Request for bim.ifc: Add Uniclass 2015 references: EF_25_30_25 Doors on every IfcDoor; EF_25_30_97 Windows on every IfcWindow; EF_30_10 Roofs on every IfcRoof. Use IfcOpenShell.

First a look at what the model holds.

```python
import ifcopenshell

model = ifcopenshell.open("bim.ifc")
print(model.schema)
print("classifications:", [c.Name for c in model.by_type("IfcClassification")])
for ifc_class in ("IfcDoor", "IfcRoof", "IfcStair", "IfcWall", "IfcWindow"):
    print(ifc_class, len(model.by_type(ifc_class)))
```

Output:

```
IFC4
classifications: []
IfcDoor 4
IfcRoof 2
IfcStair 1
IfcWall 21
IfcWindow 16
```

```python
import ifcopenshell
import ifcopenshell.api.classification

model = ifcopenshell.open("bim.ifc")

system = ifcopenshell.api.classification.add_classification(model, classification="Uniclass 2015")

codes = {
    "IfcDoor": ("EF_25_30_25", "Doors"),
    "IfcWindow": ("EF_25_30_97", "Windows"),
    "IfcRoof": ("EF_30_10", "Roofs"),
}
for ifc_class, (code, name) in codes.items():
    products = model.by_type(ifc_class)
    ifcopenshell.api.classification.add_reference(
        model, products=products, classification=system, identification=code, name=name
    )
    print(code, len(products))

model.write("bim-out.ifc")
```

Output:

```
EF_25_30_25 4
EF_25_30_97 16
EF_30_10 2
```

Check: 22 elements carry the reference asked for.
